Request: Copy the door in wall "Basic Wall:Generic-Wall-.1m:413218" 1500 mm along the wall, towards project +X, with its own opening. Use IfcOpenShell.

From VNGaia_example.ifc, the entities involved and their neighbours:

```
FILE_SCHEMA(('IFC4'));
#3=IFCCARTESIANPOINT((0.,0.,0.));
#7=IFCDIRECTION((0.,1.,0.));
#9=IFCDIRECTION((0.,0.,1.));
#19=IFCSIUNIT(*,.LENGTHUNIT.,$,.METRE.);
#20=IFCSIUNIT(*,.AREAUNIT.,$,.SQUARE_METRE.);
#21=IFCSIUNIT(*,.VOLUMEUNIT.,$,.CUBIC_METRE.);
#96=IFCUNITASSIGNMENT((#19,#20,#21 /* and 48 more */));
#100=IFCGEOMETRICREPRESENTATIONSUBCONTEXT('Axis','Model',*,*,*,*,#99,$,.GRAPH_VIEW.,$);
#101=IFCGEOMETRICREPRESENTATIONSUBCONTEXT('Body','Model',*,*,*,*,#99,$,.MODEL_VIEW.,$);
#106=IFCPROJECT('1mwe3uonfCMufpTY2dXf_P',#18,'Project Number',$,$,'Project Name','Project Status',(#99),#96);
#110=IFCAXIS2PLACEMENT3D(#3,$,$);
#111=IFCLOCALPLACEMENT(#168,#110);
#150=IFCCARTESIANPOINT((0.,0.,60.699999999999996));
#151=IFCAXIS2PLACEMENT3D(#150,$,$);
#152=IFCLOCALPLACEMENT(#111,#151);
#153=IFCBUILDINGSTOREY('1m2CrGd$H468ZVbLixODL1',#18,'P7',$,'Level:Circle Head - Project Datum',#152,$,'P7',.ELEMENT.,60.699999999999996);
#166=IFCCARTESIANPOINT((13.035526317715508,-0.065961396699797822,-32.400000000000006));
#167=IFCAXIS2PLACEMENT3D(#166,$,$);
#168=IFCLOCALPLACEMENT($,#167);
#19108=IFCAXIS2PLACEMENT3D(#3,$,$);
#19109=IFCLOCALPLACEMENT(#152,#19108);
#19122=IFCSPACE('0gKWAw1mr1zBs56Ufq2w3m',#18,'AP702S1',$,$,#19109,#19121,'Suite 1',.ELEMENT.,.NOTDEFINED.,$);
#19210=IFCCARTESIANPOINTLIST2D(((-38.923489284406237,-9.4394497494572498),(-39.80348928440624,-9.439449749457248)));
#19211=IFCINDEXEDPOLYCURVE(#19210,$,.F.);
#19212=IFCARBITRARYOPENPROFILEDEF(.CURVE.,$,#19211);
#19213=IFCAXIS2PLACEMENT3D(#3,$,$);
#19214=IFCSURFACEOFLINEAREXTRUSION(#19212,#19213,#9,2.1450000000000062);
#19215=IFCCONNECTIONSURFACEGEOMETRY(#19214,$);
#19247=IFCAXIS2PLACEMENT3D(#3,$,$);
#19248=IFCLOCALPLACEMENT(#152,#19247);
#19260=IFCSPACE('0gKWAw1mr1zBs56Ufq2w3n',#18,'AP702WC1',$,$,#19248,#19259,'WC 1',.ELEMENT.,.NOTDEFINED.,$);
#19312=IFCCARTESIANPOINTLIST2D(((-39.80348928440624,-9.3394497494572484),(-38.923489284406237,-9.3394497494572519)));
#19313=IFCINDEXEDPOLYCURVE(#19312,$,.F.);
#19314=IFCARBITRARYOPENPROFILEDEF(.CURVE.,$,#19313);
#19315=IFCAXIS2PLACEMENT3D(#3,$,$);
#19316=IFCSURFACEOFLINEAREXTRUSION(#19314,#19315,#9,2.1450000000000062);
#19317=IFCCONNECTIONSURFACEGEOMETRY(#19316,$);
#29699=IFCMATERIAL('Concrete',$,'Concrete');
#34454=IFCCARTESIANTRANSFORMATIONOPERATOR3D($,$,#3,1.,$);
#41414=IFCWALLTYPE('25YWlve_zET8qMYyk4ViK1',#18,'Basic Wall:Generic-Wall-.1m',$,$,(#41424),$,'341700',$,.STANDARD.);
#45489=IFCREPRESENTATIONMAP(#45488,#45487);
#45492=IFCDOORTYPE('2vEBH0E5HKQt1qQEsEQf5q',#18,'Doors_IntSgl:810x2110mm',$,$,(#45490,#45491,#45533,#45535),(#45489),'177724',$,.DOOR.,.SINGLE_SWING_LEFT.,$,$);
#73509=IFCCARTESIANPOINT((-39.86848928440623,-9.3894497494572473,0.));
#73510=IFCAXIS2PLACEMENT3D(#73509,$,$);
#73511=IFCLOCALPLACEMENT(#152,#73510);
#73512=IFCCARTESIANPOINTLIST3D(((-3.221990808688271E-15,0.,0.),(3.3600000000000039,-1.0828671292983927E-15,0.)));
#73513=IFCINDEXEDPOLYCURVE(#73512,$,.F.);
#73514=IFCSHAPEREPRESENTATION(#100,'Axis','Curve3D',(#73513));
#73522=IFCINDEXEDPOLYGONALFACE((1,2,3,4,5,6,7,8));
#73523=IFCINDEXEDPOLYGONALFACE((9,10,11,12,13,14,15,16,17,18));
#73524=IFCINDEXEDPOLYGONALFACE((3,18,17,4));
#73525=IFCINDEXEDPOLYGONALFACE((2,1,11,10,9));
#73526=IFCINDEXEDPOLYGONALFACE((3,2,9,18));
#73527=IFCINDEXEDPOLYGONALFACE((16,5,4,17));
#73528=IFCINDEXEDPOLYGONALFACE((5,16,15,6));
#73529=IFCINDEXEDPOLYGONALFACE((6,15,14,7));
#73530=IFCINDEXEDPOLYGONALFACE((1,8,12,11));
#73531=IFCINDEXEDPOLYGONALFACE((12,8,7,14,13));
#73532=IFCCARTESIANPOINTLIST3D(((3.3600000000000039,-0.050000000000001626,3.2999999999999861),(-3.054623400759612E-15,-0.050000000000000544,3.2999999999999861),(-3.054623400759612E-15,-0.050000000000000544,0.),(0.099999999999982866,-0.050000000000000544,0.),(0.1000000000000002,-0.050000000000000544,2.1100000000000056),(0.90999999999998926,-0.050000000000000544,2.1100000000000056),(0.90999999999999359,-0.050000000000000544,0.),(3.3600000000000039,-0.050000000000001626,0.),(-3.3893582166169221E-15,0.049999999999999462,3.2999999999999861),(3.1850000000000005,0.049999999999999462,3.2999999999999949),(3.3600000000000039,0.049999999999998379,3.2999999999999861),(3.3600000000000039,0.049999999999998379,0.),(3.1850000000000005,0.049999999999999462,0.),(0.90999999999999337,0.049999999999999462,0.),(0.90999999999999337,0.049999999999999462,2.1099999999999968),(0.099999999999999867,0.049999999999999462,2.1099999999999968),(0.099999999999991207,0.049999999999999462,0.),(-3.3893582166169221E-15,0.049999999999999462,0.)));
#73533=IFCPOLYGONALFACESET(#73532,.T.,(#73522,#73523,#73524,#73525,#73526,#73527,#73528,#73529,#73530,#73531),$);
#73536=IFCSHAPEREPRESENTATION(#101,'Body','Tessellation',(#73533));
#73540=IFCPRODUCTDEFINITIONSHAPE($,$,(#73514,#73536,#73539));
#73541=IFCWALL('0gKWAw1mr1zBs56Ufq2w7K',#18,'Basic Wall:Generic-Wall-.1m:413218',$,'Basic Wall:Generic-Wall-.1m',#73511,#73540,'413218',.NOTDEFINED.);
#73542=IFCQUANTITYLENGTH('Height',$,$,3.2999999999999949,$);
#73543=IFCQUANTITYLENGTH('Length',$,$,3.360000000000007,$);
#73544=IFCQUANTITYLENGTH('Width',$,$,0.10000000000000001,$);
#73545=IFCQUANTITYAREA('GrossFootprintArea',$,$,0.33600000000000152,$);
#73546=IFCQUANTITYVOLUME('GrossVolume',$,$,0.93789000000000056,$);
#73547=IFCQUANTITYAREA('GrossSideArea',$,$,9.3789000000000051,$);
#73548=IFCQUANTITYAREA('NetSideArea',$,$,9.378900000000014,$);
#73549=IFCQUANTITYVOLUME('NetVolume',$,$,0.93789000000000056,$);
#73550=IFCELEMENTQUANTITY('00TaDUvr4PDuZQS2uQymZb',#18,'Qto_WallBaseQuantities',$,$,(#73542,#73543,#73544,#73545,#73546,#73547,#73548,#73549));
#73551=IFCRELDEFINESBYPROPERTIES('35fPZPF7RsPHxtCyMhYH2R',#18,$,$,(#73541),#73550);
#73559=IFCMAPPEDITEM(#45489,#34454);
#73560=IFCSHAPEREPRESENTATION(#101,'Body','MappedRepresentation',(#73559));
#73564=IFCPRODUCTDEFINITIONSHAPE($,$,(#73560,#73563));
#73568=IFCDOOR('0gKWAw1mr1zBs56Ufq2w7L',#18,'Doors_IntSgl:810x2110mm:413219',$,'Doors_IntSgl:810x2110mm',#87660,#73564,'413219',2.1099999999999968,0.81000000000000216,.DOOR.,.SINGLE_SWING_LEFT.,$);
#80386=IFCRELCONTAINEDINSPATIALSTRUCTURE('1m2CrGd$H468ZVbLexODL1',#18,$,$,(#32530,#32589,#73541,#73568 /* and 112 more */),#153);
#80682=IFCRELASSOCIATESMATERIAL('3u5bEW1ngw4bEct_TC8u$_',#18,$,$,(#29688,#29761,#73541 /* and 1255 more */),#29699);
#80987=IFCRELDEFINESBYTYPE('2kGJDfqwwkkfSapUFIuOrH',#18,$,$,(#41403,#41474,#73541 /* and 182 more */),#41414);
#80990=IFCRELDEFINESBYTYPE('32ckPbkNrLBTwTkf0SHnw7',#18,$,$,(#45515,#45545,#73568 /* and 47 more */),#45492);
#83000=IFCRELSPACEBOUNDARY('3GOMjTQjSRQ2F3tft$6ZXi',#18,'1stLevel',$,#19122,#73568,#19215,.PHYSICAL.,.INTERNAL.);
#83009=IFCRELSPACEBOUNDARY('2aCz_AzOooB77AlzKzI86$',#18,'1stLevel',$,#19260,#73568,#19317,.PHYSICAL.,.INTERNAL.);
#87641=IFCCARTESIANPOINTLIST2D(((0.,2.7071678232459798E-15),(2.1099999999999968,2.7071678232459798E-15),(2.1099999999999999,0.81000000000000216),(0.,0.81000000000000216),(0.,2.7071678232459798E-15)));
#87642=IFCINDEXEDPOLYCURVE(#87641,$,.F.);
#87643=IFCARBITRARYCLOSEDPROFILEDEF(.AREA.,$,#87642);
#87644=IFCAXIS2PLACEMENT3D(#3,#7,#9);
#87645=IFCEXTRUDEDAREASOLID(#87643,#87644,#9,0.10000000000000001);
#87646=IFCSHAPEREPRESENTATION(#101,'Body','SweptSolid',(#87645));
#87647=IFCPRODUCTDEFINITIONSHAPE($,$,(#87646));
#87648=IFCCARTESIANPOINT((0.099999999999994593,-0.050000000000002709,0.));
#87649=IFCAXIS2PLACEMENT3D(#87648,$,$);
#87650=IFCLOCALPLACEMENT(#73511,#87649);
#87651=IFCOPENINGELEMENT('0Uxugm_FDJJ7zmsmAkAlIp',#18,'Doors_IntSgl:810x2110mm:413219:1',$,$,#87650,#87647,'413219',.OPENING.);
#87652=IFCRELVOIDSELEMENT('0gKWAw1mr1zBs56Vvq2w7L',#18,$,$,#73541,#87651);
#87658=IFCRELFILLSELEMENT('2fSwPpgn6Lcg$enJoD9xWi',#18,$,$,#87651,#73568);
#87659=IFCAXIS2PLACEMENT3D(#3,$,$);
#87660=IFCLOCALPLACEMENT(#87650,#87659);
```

```python
import numpy as np
import ifcopenshell
import ifcopenshell.api.feature
import ifcopenshell.api.geometry
import ifcopenshell.api.pset
import ifcopenshell.api.root
import ifcopenshell.geom
import ifcopenshell.util.element
import ifcopenshell.util.placement
import ifcopenshell.util.shape
import ifcopenshell.util.unit

model = ifcopenshell.open("VNGaia_example.ifc")
area_scale = ifcopenshell.util.unit.calculate_unit_scale(model, "AREAUNIT")
volume_scale = ifcopenshell.util.unit.calculate_unit_scale(model, "VOLUMEUNIT")
settings = ifcopenshell.geom.settings()


def volume(element):
    """Net volume in cubic metres, openings subtracted."""
    shape = ifcopenshell.geom.create_shape(settings, element)
    return ifcopenshell.util.shape.get_volume(shape.geometry)


def reuse_history(source, copy):
    """copy_class also copies each property set's owner history, people and application; keep the originals."""
    for rel in copy.IsDefinedBy:
        if rel.is_a("IfcRelDefinesByProperties") and (history := rel.RelatingPropertyDefinition.OwnerHistory):
            rel.RelatingPropertyDefinition.OwnerHistory = source.OwnerHistory
            ifcopenshell.util.element.remove_deep2(model, history)


door = model.by_guid("0gKWAw1mr1zBs56Ufq2w7L")
opening = door.FillsVoids[0].RelatingOpeningElement
wall = opening.VoidsElements[0].RelatingBuildingElement
before = volume(wall)
shift = ifcopenshell.util.placement.get_local_placement(wall.ObjectPlacement)[:3, 0] * 1.5

# copy_class copies the void relationship, type, container and properties, but no geometry.
new_opening = ifcopenshell.api.root.copy_class(model, product=opening)
new_opening.Representation = ifcopenshell.util.element.copy_deep(
    model, opening.Representation, exclude=["IfcGeometricRepresentationContext", "IfcRepresentationMap"]
)
new_opening.Name = "Doors_IntSgl:810x2110mm"
new_opening.Tag = None
reuse_history(opening, new_opening)
new_door = ifcopenshell.api.root.copy_class(model, product=door)
new_door.Representation = ifcopenshell.util.element.copy_deep(
    model, door.Representation, exclude=["IfcGeometricRepresentationContext", "IfcRepresentationMap"]
)
new_door.Name = "Doors_IntSgl:810x2110mm"
new_door.Tag = None
reuse_history(door, new_door)
ifcopenshell.api.feature.add_filling(model, opening=new_opening, element=new_door)

for old, new in ((opening, new_opening), (door, new_door)):
    matrix = ifcopenshell.util.placement.get_local_placement(old.ObjectPlacement)
    matrix[:3, 3] += shift
    ifcopenshell.api.geometry.edit_object_placement(model, product=new, matrix=matrix, is_si=False)

# The copied space boundaries still share their surfaces with the original.
for rel in new_door.ProvidesBoundaries:
    if rel.ConnectionGeometry:
        rel.ConnectionGeometry = ifcopenshell.util.element.copy_deep(model, rel.ConnectionGeometry)

# Space boundary surfaces are stored in each space's coordinates; move them too.
for rel in new_door.ProvidesBoundaries:
    if not rel.ConnectionGeometry:
        continue
    surface = rel.ConnectionGeometry.SurfaceOnRelatingElement
    space_matrix = ifcopenshell.util.placement.get_local_placement(rel.RelatingSpace.ObjectPlacement)
    point = np.array(surface.Position.Location.Coordinates) + space_matrix[:3, :3].T @ shift
    surface.Position = model.createIfcAxis2Placement3D(
        model.createIfcCartesianPoint(point.tolist()), surface.Position.Axis, surface.Position.RefDirection
    )

after = volume(wall)
thickness = 0.1  # wall thickness in metres

# Update the wall's stored quantities.
qto = model.by_id(ifcopenshell.util.element.get_pset(wall, "Qto_WallBaseQuantities", should_inherit=False)["id"])
ifcopenshell.api.pset.edit_qto(model, qto=qto, properties={
    "NetSideArea": after / thickness / area_scale,
    "NetVolume": after / volume_scale,
})

print(f"wall volume {before:.3f} -> {after:.3f} m3")

model.write("VNGaia_example-out.ifc")
```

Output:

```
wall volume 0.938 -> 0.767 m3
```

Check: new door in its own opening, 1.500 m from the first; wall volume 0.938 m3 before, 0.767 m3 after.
